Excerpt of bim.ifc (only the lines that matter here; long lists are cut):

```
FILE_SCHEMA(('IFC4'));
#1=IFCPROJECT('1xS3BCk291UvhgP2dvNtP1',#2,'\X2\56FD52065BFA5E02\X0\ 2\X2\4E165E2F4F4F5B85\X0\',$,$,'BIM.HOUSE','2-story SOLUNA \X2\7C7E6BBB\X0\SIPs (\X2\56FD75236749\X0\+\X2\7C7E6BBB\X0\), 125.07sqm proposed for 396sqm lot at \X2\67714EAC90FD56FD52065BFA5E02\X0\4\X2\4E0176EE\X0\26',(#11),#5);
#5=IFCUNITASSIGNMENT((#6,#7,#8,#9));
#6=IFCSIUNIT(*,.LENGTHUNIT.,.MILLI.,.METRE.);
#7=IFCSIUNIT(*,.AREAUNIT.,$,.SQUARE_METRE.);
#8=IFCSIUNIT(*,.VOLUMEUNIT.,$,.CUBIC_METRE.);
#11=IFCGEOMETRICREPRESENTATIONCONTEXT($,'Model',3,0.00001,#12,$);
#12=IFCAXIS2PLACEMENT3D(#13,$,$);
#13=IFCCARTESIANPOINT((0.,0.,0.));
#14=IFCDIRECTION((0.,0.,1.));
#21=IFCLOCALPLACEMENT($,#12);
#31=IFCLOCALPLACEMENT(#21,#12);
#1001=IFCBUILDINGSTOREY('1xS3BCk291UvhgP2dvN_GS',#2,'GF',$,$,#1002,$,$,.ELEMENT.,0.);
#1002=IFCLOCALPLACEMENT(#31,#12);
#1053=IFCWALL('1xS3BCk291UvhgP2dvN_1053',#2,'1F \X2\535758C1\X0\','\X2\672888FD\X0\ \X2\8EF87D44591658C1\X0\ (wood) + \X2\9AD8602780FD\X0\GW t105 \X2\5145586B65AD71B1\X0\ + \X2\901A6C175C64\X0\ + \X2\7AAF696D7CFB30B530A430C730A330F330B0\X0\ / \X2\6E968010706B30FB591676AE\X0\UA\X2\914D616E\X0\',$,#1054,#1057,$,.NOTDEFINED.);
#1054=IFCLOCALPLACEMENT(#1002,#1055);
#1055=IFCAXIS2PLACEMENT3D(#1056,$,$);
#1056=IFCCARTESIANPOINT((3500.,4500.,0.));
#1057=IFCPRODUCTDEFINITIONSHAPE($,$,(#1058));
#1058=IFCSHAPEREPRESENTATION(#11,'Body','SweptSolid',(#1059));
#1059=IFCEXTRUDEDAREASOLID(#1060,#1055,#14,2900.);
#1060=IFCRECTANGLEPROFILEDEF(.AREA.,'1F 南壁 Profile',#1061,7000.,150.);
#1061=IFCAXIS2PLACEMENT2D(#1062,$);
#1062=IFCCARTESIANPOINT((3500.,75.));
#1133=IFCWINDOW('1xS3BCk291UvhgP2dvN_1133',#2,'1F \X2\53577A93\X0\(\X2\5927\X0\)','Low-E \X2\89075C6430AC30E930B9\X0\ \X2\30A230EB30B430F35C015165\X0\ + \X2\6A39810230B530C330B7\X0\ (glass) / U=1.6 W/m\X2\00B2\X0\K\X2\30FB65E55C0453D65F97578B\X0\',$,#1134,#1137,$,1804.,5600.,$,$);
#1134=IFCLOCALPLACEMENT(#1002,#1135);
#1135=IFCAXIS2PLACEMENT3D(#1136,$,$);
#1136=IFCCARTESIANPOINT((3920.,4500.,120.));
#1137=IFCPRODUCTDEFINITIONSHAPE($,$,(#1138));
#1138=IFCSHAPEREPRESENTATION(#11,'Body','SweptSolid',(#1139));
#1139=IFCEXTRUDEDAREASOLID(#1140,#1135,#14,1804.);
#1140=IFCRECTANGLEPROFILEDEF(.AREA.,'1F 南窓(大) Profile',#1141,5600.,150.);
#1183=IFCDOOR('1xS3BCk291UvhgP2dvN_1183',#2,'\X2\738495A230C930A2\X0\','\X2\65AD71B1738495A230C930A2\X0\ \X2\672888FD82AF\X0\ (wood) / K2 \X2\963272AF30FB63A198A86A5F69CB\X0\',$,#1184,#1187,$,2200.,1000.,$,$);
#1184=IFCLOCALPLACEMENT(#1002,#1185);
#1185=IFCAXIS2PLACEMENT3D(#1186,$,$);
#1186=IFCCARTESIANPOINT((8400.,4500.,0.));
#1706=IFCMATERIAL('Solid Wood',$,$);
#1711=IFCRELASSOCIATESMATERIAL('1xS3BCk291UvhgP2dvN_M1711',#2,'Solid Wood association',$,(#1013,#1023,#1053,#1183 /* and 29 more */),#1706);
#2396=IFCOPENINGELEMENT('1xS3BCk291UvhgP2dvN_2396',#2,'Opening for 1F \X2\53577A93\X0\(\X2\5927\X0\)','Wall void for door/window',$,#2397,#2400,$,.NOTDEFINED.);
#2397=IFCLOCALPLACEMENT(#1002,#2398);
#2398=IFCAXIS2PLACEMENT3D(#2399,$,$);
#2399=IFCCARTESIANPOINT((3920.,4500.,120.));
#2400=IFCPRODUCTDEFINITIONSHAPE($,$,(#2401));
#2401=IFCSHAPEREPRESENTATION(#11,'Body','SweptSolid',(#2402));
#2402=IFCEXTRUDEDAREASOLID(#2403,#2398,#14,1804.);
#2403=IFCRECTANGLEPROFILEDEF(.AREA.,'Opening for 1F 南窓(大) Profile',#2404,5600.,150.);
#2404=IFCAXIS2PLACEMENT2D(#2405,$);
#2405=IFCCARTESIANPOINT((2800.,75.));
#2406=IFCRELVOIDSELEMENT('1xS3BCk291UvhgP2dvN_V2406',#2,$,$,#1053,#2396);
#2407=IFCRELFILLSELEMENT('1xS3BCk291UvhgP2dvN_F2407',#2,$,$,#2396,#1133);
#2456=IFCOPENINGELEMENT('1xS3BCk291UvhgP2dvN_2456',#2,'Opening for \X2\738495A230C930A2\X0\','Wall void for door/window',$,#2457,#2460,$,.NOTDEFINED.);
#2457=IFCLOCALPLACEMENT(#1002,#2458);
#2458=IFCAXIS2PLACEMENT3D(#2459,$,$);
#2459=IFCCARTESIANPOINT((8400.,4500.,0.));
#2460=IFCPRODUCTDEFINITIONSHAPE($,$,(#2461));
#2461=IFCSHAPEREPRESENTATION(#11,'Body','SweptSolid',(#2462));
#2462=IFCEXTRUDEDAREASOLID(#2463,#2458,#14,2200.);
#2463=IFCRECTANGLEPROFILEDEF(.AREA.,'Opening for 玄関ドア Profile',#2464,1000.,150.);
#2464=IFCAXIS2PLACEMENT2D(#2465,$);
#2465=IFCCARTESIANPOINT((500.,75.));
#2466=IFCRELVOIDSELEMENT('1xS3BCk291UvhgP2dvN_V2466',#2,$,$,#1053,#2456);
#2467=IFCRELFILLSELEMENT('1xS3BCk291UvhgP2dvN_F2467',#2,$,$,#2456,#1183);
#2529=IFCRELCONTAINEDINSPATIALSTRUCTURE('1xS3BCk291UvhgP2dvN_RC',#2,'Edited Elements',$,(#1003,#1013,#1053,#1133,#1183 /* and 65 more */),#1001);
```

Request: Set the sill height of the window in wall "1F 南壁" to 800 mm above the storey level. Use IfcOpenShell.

```python
import numpy as np
import ifcopenshell
import ifcopenshell.api.geometry
import ifcopenshell.geom
import ifcopenshell.util.element
import ifcopenshell.util.placement
import ifcopenshell.util.shape
import ifcopenshell.util.unit

model = ifcopenshell.open("bim.ifc")
unit_scale = ifcopenshell.util.unit.calculate_unit_scale(model)

window = model.by_guid("1xS3BCk291UvhgP2dvN_1133")
opening = window.FillsVoids[0].RelatingOpeningElement
storey = ifcopenshell.util.element.get_container(window, ifc_class="IfcBuildingStorey")
level = ifcopenshell.util.placement.get_local_placement(storey.ObjectPlacement)[2, 3]

# The opening's origin need not be at the sill, so measure its lowest point.
shape = ifcopenshell.geom.create_shape(ifcopenshell.geom.settings(), opening)
bottom = ifcopenshell.util.shape.get_shape_bottom_elevation(shape, shape.geometry) / unit_scale
dz = level + 800.0 - bottom

shift = np.array([0.0, 0.0, dz])
# The window is not placed relative to its opening, so move both.
for product in (opening, window):
    matrix = ifcopenshell.util.placement.get_local_placement(product.ObjectPlacement)
    matrix[:3, 3] += shift
    ifcopenshell.api.geometry.edit_object_placement(model, product=product, matrix=matrix, is_si=False)

print(f"moved by {dz * unit_scale:+.3f} m")

model.write("bim_v2.ifc")
```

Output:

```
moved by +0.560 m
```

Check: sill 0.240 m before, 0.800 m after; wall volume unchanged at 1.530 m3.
